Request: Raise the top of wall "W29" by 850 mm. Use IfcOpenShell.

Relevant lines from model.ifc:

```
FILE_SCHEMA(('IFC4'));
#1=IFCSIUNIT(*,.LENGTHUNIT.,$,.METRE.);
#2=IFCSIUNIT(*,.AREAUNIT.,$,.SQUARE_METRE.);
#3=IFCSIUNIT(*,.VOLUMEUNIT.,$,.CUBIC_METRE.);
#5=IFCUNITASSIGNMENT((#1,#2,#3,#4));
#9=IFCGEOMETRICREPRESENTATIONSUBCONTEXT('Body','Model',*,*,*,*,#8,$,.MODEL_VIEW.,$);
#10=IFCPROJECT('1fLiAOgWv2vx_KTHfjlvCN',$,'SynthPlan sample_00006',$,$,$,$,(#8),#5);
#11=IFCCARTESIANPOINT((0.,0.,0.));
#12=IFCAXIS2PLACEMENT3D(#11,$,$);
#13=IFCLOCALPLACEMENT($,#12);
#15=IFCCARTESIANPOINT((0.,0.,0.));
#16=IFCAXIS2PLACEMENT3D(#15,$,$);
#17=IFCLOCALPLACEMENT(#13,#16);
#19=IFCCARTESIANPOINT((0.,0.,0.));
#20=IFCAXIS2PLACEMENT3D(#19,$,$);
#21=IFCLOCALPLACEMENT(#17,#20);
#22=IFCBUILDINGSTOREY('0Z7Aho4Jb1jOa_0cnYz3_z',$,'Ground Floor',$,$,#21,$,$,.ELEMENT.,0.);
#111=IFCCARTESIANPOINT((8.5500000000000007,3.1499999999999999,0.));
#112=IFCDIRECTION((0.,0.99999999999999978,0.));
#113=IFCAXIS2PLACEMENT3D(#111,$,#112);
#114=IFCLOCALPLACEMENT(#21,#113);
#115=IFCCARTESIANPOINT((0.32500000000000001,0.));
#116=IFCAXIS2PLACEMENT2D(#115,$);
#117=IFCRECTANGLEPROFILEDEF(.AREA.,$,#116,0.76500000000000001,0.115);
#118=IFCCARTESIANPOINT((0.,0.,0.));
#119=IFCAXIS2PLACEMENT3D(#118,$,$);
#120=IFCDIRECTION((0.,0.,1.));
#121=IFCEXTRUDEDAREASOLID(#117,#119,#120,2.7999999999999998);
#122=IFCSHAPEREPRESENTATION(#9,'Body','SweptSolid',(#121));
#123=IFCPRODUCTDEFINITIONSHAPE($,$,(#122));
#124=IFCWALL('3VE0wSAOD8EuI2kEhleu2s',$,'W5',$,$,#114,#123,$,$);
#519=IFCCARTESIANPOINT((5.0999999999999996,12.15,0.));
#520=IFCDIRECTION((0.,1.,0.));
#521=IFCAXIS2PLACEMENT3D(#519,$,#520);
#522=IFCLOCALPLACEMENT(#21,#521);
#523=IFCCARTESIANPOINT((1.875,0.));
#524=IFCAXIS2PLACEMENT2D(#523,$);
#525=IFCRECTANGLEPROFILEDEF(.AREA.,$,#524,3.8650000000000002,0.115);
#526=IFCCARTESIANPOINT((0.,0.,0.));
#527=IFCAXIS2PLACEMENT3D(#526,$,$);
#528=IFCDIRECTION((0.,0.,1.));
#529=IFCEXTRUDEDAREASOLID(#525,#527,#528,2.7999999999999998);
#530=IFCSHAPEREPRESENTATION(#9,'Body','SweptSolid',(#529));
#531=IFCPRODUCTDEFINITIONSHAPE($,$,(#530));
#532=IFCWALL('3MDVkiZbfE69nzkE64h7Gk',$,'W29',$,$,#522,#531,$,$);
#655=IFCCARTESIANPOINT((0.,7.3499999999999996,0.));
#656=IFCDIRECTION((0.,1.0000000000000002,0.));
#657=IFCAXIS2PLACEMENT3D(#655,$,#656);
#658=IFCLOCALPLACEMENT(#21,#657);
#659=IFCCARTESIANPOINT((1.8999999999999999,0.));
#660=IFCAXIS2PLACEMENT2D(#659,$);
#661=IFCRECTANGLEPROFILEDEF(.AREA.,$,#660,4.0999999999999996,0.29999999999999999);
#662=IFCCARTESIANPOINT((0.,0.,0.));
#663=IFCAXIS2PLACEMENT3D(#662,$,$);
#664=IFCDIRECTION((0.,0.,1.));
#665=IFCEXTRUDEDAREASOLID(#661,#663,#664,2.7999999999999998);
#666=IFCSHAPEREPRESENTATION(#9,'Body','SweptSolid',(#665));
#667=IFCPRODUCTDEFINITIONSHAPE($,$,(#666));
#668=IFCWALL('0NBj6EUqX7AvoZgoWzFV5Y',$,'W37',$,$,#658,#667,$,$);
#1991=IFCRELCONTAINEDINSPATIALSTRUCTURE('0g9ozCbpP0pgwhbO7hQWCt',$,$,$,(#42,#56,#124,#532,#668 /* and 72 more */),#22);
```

```python
import ifcopenshell
import ifcopenshell.geom
import ifcopenshell.util.representation
import ifcopenshell.util.shape
import ifcopenshell.util.unit

model = ifcopenshell.open("model.ifc")
unit_scale = ifcopenshell.util.unit.calculate_unit_scale(model)
settings = ifcopenshell.geom.settings()


def volume(element):
    """Net volume in cubic metres, openings subtracted."""
    shape = ifcopenshell.geom.create_shape(settings, element)
    return ifcopenshell.util.shape.get_volume(shape.geometry)


wall = model.by_guid("3MDVkiZbfE69nzkE64h7Gk")
before = volume(wall)

body = ifcopenshell.util.representation.get_representation(wall, "Model", "Body")
solid = body.Items[0]
old_height = solid.Depth
solid.Depth += 0.85 / unit_scale
after = volume(wall)

print(f"height {old_height:g} -> {solid.Depth:g}, volume {before:.3f} -> {after:.3f} m3")

model.write("model-out.ifc")
```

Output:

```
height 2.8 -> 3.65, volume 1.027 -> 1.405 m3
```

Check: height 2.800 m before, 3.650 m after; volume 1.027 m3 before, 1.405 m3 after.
